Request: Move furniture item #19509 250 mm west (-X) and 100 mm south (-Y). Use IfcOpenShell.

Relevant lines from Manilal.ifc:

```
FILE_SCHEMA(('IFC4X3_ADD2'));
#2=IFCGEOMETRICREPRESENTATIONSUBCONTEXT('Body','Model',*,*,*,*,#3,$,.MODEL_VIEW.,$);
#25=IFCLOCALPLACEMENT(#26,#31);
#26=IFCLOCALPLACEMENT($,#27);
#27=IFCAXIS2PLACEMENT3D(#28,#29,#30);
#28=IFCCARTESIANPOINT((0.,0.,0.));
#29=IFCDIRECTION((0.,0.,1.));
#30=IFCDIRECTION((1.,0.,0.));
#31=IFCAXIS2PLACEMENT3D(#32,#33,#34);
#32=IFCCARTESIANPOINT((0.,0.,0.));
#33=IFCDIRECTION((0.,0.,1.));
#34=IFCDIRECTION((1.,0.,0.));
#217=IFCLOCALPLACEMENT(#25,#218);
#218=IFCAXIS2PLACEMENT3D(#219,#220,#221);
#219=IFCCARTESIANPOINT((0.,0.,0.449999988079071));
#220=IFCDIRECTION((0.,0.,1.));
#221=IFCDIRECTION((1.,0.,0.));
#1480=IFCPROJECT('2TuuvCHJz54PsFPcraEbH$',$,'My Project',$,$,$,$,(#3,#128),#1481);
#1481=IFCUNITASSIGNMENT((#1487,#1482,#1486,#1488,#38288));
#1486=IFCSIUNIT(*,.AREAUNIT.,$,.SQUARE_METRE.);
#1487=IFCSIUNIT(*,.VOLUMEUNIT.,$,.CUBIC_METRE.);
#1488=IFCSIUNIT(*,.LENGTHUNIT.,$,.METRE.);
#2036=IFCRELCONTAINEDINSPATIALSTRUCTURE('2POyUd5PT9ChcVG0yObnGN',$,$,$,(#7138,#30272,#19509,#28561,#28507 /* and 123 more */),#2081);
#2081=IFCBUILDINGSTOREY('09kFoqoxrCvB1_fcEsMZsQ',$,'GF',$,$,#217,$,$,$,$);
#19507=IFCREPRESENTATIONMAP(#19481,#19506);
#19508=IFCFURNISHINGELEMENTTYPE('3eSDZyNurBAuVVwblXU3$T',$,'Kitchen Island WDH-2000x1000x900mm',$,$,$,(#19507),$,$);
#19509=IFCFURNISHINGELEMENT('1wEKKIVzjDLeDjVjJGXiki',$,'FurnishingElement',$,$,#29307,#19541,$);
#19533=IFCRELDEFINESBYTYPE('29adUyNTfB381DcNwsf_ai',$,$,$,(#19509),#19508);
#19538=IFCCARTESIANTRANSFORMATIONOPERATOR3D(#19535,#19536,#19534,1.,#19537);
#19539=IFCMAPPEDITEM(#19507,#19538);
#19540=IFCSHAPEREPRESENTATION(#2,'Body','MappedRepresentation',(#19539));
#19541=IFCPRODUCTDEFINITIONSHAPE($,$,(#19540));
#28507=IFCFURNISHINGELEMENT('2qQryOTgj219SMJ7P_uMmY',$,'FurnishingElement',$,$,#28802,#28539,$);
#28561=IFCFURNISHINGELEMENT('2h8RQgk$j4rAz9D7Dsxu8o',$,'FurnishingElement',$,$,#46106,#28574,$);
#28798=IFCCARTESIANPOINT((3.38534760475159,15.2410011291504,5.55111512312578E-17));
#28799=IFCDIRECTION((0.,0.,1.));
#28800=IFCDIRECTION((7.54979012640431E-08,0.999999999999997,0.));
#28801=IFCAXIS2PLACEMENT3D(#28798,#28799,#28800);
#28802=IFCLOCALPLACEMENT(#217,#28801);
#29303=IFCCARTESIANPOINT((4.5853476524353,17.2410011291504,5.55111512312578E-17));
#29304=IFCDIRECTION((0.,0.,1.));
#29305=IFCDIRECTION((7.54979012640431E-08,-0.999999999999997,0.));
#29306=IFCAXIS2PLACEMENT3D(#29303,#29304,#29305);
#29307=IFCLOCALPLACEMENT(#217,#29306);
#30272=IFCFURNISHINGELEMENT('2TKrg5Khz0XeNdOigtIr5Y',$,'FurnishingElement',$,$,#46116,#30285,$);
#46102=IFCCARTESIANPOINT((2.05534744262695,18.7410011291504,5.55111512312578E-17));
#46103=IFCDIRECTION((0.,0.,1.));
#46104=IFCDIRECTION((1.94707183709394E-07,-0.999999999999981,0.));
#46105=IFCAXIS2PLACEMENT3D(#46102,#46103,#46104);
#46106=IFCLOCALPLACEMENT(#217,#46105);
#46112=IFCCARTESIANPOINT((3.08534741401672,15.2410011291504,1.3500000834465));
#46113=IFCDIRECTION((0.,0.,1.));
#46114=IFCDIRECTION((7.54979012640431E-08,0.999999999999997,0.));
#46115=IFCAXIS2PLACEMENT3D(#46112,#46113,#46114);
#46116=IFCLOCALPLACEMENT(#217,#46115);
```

```python
import ifcopenshell
import ifcopenshell.api.geometry
import ifcopenshell.util.placement
import ifcopenshell.util.unit

model = ifcopenshell.open("Manilal.ifc")
unit_scale = ifcopenshell.util.unit.calculate_unit_scale(model)

item = model.by_guid("1wEKKIVzjDLeDjVjJGXiki")
matrix = ifcopenshell.util.placement.get_local_placement(item.ObjectPlacement)
matrix[0, 3] -= 0.25 / unit_scale
matrix[1, 3] -= 0.1 / unit_scale
ifcopenshell.api.geometry.edit_object_placement(model, product=item, matrix=matrix, is_si=False)

print(ifcopenshell.util.placement.get_local_placement(item.ObjectPlacement).round(3) + 0.0)

model.write("Manilal-out.ifc")
```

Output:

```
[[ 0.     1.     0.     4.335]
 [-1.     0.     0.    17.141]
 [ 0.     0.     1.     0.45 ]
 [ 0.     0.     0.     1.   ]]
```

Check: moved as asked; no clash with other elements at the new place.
